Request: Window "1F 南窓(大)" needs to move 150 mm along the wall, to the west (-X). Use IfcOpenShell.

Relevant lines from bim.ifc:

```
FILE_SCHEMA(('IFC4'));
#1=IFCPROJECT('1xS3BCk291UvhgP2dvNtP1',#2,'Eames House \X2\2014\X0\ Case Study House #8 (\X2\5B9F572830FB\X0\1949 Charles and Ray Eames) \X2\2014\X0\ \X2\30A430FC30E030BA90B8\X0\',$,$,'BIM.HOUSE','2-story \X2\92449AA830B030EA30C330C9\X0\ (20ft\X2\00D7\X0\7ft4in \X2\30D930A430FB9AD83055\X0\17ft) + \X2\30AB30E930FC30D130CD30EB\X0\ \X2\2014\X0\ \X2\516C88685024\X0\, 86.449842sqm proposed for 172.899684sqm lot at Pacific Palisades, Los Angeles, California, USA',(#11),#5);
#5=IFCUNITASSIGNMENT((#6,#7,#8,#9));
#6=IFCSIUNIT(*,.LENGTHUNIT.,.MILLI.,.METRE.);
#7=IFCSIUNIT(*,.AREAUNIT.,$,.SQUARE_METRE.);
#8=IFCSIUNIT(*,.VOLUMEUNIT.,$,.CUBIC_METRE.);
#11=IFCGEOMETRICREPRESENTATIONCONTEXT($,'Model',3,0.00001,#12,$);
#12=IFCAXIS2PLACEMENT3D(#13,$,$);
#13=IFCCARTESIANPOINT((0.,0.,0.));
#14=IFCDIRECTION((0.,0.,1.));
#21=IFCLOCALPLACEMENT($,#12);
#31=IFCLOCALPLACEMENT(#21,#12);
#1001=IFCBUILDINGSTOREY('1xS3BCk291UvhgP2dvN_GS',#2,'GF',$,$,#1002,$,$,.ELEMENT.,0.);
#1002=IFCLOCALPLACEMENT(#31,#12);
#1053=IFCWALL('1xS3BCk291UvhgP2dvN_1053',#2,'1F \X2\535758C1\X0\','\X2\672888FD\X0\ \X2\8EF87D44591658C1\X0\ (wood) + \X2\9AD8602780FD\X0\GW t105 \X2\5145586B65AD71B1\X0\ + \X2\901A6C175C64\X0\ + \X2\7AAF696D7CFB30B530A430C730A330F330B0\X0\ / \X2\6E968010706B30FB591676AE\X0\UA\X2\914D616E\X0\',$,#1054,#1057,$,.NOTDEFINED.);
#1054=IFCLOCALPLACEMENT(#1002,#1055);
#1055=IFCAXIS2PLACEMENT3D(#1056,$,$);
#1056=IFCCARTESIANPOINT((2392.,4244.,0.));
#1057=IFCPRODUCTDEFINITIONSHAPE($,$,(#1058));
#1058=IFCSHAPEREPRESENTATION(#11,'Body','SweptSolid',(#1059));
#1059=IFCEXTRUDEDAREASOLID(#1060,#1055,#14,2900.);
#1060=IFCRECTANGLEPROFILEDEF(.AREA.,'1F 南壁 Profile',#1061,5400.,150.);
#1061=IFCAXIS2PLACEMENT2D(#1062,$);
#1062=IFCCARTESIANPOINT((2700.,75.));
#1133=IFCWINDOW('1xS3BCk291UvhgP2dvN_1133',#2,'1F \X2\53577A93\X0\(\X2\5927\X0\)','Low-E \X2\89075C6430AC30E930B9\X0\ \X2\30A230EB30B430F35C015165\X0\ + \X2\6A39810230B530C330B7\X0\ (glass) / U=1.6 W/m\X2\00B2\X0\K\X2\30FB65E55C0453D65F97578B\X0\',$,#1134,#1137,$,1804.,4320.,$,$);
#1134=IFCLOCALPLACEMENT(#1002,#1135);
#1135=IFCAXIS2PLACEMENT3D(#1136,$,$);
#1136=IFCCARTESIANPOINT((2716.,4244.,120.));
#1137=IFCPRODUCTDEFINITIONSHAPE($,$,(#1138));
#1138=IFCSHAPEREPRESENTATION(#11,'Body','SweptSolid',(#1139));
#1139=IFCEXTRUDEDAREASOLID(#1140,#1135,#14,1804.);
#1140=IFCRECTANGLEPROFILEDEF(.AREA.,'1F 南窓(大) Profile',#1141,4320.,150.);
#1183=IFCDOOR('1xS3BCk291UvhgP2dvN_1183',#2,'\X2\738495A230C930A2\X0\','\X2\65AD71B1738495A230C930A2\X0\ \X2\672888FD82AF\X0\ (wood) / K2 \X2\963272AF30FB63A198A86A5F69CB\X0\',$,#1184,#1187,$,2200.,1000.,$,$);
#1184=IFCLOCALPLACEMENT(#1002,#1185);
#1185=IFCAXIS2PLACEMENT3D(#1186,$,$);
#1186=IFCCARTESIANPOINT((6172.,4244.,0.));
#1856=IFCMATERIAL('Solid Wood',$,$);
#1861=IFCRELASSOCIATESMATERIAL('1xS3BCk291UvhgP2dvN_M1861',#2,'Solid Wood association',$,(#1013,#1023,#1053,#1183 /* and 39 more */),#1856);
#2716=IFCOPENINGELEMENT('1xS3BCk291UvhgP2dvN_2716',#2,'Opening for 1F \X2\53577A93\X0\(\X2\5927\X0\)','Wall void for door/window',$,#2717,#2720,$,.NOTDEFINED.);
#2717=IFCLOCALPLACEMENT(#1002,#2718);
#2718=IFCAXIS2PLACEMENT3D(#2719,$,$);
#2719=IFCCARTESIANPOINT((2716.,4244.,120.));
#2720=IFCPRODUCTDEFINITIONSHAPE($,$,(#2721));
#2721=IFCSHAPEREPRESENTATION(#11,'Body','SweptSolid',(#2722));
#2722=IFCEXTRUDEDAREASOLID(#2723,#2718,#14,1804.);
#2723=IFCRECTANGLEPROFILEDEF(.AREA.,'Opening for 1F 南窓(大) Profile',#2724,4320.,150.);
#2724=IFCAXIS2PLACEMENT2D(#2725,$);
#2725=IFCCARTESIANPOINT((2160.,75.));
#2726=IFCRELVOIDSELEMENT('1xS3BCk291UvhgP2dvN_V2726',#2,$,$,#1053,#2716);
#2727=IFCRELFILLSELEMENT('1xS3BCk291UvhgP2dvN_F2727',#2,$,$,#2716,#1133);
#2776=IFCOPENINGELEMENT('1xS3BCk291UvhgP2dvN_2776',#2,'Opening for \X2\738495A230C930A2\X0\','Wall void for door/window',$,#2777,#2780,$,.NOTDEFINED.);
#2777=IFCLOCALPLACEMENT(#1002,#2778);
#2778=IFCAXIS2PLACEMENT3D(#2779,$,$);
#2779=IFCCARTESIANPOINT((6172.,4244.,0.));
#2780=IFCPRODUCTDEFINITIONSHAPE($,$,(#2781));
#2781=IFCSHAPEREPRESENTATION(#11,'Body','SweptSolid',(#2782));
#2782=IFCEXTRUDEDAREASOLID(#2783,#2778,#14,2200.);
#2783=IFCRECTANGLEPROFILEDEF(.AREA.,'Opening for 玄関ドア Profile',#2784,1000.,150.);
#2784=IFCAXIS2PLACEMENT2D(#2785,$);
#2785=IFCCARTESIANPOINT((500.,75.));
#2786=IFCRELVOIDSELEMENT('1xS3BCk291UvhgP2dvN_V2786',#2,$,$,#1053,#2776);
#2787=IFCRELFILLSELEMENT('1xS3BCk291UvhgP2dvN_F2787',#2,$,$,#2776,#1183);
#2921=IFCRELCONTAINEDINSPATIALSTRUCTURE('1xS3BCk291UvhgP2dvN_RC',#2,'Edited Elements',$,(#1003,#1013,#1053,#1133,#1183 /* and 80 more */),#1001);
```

```python
import ifcopenshell
import ifcopenshell.api.geometry
import ifcopenshell.util.placement

model = ifcopenshell.open("bim.ifc")

window = model.by_id(1133)
opening = window.FillsVoids[0].RelatingOpeningElement
wall = opening.VoidsElements[0].RelatingBuildingElement

wall_matrix = ifcopenshell.util.placement.get_local_placement(wall.ObjectPlacement)
shift = wall_matrix[:3, 0] * -150.0
before = ifcopenshell.util.placement.get_local_placement(window.ObjectPlacement)[:3, 3].copy()

# The window is not placed relative to its opening, so move both.
for product in (opening, window):
    matrix = ifcopenshell.util.placement.get_local_placement(product.ObjectPlacement)
    matrix[:3, 3] += shift
    ifcopenshell.api.geometry.edit_object_placement(model, product=product, matrix=matrix, is_si=False)

after = ifcopenshell.util.placement.get_local_placement(window.ObjectPlacement)[:3, 3]
print("window moved by", (after - before).round(3) + 0.0)

model.write("bim-out.ifc")
```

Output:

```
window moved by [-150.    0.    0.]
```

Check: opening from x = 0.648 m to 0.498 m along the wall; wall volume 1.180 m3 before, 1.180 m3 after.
